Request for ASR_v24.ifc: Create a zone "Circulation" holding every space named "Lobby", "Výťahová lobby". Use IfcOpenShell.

First a look at what the model holds.

```python
import ifcopenshell

model = ifcopenshell.open("ASR_v24.ifc")
print(model.schema)
seen = {}
for space in model.by_type("IfcSpace"):
    seen[space.LongName] = seen.get(space.LongName, 0) + 1
for name, count in sorted(seen.items(), key=str):
    print(count, "x", name)
print("zones:", [z.Name for z in model.by_type("IfcZone")][:20])
```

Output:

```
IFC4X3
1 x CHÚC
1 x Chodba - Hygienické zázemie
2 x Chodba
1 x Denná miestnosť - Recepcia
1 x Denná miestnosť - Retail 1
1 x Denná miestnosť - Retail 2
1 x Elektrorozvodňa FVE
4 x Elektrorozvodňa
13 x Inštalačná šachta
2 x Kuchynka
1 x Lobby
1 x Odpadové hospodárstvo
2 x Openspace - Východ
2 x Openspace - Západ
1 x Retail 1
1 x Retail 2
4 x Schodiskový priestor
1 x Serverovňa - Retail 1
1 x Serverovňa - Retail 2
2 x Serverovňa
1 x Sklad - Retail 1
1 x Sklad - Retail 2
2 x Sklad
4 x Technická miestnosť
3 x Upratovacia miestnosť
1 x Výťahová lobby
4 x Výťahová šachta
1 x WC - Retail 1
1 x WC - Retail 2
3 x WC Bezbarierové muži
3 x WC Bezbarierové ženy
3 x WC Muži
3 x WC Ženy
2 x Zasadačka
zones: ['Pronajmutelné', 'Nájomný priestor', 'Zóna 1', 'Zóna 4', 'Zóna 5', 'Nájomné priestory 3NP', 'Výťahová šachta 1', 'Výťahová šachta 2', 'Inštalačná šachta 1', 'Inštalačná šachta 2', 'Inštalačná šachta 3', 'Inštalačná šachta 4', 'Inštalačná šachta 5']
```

```python
import ifcopenshell
import ifcopenshell.api.group
import ifcopenshell.api.root

model = ifcopenshell.open("ASR_v24.ifc")

names = {"Lobby", "Výťahová lobby"}
spaces = [s for s in model.by_type("IfcSpace") if s.LongName in names]

zone = ifcopenshell.api.root.create_entity(model, ifc_class="IfcZone", name="Circulation")
ifcopenshell.api.group.assign_group(model, products=spaces, group=zone)
print(len(spaces), "spaces in", zone.Name)

model.write("ASR_v24_edited.ifc")
```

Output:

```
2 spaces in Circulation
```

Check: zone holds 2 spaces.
